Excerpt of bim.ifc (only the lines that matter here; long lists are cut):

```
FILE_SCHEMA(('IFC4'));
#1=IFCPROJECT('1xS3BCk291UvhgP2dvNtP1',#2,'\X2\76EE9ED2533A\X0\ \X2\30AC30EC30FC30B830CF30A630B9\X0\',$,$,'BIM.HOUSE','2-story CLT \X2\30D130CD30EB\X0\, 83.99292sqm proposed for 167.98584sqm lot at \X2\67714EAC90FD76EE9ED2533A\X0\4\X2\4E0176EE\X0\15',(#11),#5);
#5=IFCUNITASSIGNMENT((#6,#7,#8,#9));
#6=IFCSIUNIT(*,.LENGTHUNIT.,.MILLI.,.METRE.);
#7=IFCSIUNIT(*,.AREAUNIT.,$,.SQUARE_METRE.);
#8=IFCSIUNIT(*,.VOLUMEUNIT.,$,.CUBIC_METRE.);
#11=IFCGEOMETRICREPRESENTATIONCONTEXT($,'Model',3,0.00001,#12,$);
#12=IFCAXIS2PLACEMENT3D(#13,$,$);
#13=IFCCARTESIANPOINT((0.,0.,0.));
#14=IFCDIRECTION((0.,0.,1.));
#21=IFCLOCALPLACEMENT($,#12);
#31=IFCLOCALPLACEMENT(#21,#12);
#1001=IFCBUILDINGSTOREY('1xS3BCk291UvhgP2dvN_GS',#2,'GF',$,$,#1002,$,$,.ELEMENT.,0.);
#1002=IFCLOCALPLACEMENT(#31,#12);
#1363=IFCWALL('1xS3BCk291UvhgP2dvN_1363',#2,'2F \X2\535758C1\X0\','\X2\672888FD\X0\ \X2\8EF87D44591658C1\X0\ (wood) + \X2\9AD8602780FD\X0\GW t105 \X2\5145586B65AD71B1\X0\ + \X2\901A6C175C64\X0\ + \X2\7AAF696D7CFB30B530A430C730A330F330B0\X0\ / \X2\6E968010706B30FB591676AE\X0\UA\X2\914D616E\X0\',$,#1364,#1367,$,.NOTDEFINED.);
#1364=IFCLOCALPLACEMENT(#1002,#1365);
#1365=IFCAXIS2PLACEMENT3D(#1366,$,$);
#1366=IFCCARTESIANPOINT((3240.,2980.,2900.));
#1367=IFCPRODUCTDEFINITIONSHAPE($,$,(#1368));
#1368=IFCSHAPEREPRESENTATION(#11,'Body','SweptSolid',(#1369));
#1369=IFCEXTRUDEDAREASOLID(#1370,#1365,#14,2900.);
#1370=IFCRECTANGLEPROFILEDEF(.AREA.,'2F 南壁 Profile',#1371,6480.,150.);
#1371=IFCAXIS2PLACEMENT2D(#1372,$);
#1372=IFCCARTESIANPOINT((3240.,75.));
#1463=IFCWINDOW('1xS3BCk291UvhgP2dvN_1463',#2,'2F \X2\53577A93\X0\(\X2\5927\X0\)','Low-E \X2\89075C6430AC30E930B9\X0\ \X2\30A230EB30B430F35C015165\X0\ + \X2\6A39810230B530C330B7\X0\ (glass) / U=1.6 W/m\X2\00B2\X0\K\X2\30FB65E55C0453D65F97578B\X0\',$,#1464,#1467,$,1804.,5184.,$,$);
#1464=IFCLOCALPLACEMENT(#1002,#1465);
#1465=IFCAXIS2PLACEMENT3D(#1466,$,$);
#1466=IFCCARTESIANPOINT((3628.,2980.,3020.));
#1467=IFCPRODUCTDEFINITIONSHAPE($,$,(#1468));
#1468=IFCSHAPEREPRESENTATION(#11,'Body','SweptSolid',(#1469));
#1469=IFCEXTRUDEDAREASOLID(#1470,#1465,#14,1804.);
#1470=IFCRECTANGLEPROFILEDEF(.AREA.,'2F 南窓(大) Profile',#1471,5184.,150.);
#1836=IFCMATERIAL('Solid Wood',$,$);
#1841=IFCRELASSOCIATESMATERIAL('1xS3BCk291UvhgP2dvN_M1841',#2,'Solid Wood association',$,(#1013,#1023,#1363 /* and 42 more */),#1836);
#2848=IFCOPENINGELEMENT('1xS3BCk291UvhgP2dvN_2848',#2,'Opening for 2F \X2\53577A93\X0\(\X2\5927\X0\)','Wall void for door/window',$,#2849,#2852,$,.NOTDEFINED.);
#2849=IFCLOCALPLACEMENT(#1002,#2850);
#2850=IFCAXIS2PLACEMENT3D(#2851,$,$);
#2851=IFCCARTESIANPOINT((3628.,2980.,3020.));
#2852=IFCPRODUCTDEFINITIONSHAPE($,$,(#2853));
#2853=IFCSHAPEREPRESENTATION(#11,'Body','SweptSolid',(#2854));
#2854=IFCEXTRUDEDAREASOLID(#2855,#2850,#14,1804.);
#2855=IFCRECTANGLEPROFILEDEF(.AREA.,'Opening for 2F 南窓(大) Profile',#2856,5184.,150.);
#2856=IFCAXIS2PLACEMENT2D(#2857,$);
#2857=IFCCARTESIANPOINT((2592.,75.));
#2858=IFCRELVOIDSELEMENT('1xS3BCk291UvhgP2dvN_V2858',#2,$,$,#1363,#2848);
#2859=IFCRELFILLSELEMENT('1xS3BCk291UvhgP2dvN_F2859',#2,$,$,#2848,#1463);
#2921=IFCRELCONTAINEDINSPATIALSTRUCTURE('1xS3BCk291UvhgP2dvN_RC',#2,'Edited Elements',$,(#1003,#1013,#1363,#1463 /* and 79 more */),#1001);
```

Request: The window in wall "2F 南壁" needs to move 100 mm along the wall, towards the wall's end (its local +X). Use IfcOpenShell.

```python
import ifcopenshell
import ifcopenshell.api.geometry
import ifcopenshell.util.placement
import ifcopenshell.util.unit

model = ifcopenshell.open("bim.ifc")
unit_scale = ifcopenshell.util.unit.calculate_unit_scale(model)

window = model.by_id(1463)
opening = window.FillsVoids[0].RelatingOpeningElement
wall = opening.VoidsElements[0].RelatingBuildingElement

wall_matrix = ifcopenshell.util.placement.get_local_placement(wall.ObjectPlacement)
shift = wall_matrix[:3, 0] * 0.1 / unit_scale
before = ifcopenshell.util.placement.get_local_placement(window.ObjectPlacement)[:3, 3].copy()

# The window is not placed relative to its opening, so move both.
for product in (opening, window):
    matrix = ifcopenshell.util.placement.get_local_placement(product.ObjectPlacement)
    matrix[:3, 3] += shift
    ifcopenshell.api.geometry.edit_object_placement(model, product=product, matrix=matrix, is_si=False)

after = ifcopenshell.util.placement.get_local_placement(window.ObjectPlacement)[:3, 3]
print("window moved by", (after - before).round(3) + 0.0)

model.write("bim_rev.ifc")
```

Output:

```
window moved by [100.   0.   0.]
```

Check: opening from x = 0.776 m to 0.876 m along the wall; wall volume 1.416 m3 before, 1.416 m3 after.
